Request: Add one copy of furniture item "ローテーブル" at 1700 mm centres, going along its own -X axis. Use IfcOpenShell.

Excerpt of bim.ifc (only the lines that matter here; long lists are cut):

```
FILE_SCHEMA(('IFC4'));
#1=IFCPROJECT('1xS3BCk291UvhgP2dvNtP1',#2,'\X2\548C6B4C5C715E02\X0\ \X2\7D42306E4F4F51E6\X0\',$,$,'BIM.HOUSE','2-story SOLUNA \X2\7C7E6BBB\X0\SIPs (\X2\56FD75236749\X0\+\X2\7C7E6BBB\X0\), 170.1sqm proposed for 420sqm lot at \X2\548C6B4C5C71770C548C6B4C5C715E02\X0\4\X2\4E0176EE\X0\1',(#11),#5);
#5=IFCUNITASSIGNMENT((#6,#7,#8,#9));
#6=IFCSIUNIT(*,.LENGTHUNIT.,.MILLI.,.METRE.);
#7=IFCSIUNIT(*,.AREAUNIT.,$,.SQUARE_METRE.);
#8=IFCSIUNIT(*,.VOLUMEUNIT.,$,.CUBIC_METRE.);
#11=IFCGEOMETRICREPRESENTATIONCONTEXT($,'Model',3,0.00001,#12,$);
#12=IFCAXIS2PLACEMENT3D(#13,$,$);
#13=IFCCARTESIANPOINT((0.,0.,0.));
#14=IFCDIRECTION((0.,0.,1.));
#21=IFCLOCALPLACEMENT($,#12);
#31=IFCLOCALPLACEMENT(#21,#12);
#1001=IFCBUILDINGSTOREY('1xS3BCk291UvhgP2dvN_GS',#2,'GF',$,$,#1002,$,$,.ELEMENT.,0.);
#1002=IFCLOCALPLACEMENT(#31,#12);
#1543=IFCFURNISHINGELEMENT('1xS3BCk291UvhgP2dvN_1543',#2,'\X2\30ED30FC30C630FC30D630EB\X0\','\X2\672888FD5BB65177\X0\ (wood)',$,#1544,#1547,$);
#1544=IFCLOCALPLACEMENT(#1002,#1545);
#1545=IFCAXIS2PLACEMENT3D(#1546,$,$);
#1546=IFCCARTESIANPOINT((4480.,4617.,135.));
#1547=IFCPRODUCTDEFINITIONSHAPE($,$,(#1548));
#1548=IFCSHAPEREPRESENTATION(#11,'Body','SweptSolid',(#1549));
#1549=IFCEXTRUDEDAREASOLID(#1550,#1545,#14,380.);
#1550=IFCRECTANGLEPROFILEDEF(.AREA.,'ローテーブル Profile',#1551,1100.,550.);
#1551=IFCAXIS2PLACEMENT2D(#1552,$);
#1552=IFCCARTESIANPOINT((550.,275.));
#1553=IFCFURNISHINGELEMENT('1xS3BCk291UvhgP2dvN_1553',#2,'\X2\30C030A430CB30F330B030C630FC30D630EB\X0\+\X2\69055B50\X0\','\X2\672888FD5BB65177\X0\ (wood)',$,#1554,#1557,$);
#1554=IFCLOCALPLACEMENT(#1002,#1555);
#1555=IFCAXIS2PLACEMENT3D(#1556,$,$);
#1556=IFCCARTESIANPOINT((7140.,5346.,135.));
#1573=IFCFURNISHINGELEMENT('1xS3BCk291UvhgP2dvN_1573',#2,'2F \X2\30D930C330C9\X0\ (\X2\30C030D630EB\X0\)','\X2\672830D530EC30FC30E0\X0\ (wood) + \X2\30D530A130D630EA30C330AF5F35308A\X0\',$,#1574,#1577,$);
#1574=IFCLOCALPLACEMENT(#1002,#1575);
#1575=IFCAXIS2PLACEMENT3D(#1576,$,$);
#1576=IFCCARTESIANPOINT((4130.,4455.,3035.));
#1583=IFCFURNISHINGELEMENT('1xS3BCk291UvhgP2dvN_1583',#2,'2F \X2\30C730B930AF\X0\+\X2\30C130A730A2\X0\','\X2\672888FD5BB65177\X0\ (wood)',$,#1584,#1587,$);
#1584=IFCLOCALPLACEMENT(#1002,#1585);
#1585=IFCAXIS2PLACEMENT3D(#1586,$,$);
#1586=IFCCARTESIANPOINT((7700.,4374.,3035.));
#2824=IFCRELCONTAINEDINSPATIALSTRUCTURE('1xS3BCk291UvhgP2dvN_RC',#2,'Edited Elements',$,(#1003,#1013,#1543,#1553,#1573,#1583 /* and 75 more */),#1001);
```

```python
import ifcopenshell
import ifcopenshell.api.geometry
import ifcopenshell.api.root
import ifcopenshell.util.element
import ifcopenshell.util.placement

model = ifcopenshell.open("bim.ifc")


def reuse_history(source, copy):
    """copy_class also copies each property set's owner history, people and application; keep the originals."""
    for rel in copy.IsDefinedBy:
        if rel.is_a("IfcRelDefinesByProperties") and (history := rel.RelatingPropertyDefinition.OwnerHistory):
            rel.RelatingPropertyDefinition.OwnerHistory = source.OwnerHistory
            ifcopenshell.util.element.remove_deep2(model, history)


source = model.by_guid("1xS3BCk291UvhgP2dvN_1543")
base = ifcopenshell.util.placement.get_local_placement(source.ObjectPlacement)
step = -base[:3, 0] * 1700.0

for i in range(1, 2):
    copy = ifcopenshell.api.root.copy_class(model, product=source)
    copy.Representation = ifcopenshell.util.element.copy_deep(
        model, source.Representation, exclude=["IfcGeometricRepresentationContext", "IfcRepresentationMap"]
    )
    reuse_history(source, copy)
    matrix = base.copy()
    matrix[:3, 3] += i * step
    print("added at", matrix[:3, 3].round(3) + 0.0)
    ifcopenshell.api.geometry.edit_object_placement(model, product=copy, matrix=matrix, is_si=False)

model.write("bim_updated.ifc")
```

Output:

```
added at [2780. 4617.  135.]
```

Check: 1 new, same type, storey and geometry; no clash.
